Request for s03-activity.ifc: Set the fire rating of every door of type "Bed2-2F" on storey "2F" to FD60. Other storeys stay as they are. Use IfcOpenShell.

First a look at what the model holds.

```python
import ifcopenshell
import ifcopenshell.util.element

model = ifcopenshell.open("s03-activity.ifc")
print(model.schema)
storey = next(s for s in model.by_type("IfcBuildingStorey") if s.Name == "2F")
doors = [e for e in ifcopenshell.util.element.get_decomposition(storey) if e.is_a("IfcDoor")]
seen = {}
for e in doors:
    element_type = ifcopenshell.util.element.get_type(e)
    key = (element_type.Name if element_type != e and element_type else None, ifcopenshell.util.element.get_pset(e, "Pset_DoorCommon", "FireRating"))
    seen[key] = seen.get(key, 0) + 1
for (name, value), count in sorted(seen.items(), key=str):
    print(count, "x", name, "|", value)
```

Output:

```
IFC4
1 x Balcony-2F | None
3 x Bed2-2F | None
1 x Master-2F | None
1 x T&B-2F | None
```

```python
import ifcopenshell
import ifcopenshell.api.pset
import ifcopenshell.util.element

model = ifcopenshell.open("s03-activity.ifc")

storey = next(s for s in model.by_type("IfcBuildingStorey") if s.Name == "2F")
doors = [e for e in ifcopenshell.util.element.get_decomposition(storey) if e.is_a("IfcDoor")]

count = 0
for e in doors:
    element_type = ifcopenshell.util.element.get_type(e)
    if element_type in (None, e) or element_type.Name != "Bed2-2F":
        continue
    # add_pset returns the element's existing set when there is one.
    pset = ifcopenshell.api.pset.add_pset(model, product=e, name="Pset_DoorCommon")
    ifcopenshell.api.pset.edit_pset(model, pset=pset, properties={"FireRating": "FD60"})
    count += 1

print(count, "doors updated")

model.write("s03-activity_edited.ifc")
```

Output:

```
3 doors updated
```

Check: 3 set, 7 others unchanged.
